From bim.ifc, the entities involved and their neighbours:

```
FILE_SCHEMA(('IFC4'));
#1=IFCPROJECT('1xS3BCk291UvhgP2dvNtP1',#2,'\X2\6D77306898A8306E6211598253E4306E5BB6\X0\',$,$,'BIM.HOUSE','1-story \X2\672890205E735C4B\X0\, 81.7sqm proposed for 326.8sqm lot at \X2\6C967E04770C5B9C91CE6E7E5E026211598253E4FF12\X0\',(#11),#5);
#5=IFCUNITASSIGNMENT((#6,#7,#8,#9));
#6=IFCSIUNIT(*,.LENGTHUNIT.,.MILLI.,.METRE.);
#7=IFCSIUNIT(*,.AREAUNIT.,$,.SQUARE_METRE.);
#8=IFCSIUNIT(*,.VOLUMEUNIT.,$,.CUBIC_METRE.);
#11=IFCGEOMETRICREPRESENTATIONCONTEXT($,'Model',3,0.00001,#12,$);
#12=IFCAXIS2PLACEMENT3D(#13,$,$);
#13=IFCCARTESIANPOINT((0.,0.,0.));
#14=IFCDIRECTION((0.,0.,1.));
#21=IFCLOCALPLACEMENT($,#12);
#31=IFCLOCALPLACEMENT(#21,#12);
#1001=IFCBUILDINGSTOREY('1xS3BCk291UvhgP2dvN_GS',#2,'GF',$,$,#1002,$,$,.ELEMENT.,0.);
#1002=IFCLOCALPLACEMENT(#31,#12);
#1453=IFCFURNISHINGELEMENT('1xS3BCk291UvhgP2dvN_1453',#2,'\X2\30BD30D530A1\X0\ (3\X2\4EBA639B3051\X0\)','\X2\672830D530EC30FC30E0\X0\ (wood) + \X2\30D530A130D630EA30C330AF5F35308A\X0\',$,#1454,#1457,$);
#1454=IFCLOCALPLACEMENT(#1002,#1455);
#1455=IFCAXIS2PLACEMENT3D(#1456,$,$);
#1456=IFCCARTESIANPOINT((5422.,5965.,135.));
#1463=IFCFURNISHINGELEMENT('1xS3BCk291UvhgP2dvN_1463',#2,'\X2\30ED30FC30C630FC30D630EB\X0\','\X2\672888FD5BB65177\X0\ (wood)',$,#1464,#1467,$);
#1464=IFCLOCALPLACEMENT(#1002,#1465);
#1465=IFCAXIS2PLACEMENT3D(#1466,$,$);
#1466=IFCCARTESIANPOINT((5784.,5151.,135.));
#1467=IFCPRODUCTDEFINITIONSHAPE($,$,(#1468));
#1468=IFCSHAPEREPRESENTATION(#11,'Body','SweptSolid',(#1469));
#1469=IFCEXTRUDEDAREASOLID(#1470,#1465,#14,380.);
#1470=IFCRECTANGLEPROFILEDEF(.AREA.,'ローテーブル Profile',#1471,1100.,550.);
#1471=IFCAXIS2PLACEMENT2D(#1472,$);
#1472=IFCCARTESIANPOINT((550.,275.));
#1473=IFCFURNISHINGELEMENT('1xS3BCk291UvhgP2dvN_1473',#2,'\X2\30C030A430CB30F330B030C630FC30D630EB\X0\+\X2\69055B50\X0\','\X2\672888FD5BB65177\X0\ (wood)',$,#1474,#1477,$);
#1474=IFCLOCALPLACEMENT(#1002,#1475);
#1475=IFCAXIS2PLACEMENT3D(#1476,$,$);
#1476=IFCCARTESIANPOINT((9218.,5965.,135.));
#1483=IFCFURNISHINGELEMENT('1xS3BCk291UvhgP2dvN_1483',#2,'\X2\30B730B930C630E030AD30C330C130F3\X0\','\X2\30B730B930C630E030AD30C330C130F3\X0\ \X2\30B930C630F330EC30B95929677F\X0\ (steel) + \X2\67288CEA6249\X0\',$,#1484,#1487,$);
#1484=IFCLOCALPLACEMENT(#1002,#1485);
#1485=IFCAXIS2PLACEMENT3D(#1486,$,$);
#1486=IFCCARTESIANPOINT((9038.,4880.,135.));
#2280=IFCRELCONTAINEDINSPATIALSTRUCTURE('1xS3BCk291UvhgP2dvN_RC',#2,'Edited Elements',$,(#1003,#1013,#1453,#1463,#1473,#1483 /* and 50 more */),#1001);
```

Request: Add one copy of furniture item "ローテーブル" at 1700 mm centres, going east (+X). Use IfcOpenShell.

```python
import numpy as np
import ifcopenshell
import ifcopenshell.api.geometry
import ifcopenshell.api.root
import ifcopenshell.util.element
import ifcopenshell.util.placement

model = ifcopenshell.open("bim.ifc")


def reuse_history(source, copy):
    """copy_class also copies each property set's owner history, people and application; keep the originals."""
    for rel in copy.IsDefinedBy:
        if rel.is_a("IfcRelDefinesByProperties") and (history := rel.RelatingPropertyDefinition.OwnerHistory):
            rel.RelatingPropertyDefinition.OwnerHistory = source.OwnerHistory
            ifcopenshell.util.element.remove_deep2(model, history)


source = model.by_guid("1xS3BCk291UvhgP2dvN_1463")
base = ifcopenshell.util.placement.get_local_placement(source.ObjectPlacement)
step = np.array([1.0, 0.0, 0.0]) * 1700.0

for i in range(1, 2):
    copy = ifcopenshell.api.root.copy_class(model, product=source)
    copy.Representation = ifcopenshell.util.element.copy_deep(
        model, source.Representation, exclude=["IfcGeometricRepresentationContext", "IfcRepresentationMap"]
    )
    reuse_history(source, copy)
    matrix = base.copy()
    matrix[:3, 3] += i * step
    print("added at", matrix[:3, 3].round(3) + 0.0)
    ifcopenshell.api.geometry.edit_object_placement(model, product=copy, matrix=matrix, is_si=False)

model.write("bim_v2.ifc")
```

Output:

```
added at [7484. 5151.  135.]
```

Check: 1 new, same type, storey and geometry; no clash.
